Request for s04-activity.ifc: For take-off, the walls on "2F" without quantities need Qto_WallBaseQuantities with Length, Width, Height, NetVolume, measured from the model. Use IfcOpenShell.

First a look at what the model holds.

```python
import ifcopenshell
import ifcopenshell.util.element
import ifcopenshell.util.unit

model = ifcopenshell.open("s04-activity.ifc")
print(model.schema)
for unit_type in ("LENGTHUNIT", "AREAUNIT", "VOLUMEUNIT"):
    print(unit_type, ifcopenshell.util.unit.calculate_unit_scale(model, unit_type))
storey = next(s for s in model.by_type("IfcBuildingStorey") if s.Name == "2F")
walls = [e for e in ifcopenshell.util.element.get_decomposition(storey) if e.is_a("IfcWall")]
for e in sorted(walls, key=lambda e: e.id()):
    print(e.id(), e.is_a(), e.Name, list(ifcopenshell.util.element.get_psets(e, qtos_only=True)), sep=" | ")
```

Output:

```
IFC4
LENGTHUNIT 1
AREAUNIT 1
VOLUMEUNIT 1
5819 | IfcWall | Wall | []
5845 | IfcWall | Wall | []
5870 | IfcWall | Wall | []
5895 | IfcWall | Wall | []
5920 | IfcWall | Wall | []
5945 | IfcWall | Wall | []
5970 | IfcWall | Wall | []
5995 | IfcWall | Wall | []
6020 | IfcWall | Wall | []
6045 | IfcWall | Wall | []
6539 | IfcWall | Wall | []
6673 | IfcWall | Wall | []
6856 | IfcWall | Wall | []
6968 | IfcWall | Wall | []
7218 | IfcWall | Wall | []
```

```python
import ifcopenshell
import ifcopenshell.api.pset
import ifcopenshell.geom
import ifcopenshell.util.element
import ifcopenshell.util.shape
import ifcopenshell.util.unit

model = ifcopenshell.open("s04-activity.ifc")
unit_scale = ifcopenshell.util.unit.calculate_unit_scale(model)
volume_scale = ifcopenshell.util.unit.calculate_unit_scale(model, "VOLUMEUNIT")
settings = ifcopenshell.geom.settings()

storey = next(s for s in model.by_type("IfcBuildingStorey") if s.Name == "2F")
walls = [e for e in ifcopenshell.util.element.get_decomposition(storey) if e.is_a("IfcWall")]

for e in sorted(walls, key=lambda e: e.id()):
    if ifcopenshell.util.element.get_psets(e, qtos_only=True, should_inherit=False):
        continue
    # Geometry comes back in metres, in the element's own axes.
    shape = ifcopenshell.geom.create_shape(settings, e)
    values = {
        "Length": ifcopenshell.util.shape.get_x(shape.geometry) / unit_scale,
        "Width": ifcopenshell.util.shape.get_y(shape.geometry) / unit_scale,
        "Height": ifcopenshell.util.shape.get_z(shape.geometry) / unit_scale,
        "NetVolume": ifcopenshell.util.shape.get_volume(shape.geometry) / volume_scale,
    }
    qto = ifcopenshell.api.pset.add_qto(model, product=e, name="Qto_WallBaseQuantities")
    ifcopenshell.api.pset.edit_qto(model, qto=qto, properties=values)
    print(e.id(), {k: round(v, 3) for k, v in values.items()})

model.write("s04-activity_v2.ifc")
```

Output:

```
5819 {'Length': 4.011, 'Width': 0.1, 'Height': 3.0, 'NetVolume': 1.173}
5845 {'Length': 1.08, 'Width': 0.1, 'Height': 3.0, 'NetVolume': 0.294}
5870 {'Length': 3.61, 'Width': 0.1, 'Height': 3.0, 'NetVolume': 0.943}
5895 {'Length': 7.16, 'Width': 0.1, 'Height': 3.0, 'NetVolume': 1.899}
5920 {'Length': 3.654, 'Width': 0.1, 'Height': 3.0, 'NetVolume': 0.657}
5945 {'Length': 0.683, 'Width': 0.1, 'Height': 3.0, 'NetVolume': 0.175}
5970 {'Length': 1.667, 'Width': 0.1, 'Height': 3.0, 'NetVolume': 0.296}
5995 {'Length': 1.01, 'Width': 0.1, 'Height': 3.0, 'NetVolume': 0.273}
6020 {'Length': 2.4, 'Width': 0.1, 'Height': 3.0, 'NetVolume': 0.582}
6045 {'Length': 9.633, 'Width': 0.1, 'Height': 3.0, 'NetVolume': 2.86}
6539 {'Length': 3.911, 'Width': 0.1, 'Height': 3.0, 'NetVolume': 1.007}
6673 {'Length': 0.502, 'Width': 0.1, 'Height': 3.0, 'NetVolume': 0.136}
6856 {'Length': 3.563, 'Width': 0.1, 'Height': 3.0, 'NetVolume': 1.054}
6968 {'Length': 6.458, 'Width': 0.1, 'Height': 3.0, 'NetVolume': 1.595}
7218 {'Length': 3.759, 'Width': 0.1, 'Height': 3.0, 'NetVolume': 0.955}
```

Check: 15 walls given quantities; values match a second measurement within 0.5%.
